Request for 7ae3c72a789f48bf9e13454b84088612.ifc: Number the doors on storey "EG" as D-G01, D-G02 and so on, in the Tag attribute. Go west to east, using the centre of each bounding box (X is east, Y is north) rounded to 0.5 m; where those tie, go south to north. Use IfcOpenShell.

First a look at what the model holds.

```python
import ifcopenshell
import ifcopenshell.util.element
import ifcopenshell.util.placement

model = ifcopenshell.open("7ae3c72a789f48bf9e13454b84088612.ifc")
print(model.schema)
storey = next(s for s in model.by_type("IfcBuildingStorey") if s.Name == "EG")
doors = [e for e in ifcopenshell.util.element.get_decomposition(storey) if e.is_a("IfcDoor")]
for e in sorted(doors, key=lambda e: e.id()):
    origin = ifcopenshell.util.placement.get_local_placement(e.ObjectPlacement)[:3, 3]
    print(e.id(), e.Tag, e.Name, origin.round(2) + 0.0, sep=" | ")
```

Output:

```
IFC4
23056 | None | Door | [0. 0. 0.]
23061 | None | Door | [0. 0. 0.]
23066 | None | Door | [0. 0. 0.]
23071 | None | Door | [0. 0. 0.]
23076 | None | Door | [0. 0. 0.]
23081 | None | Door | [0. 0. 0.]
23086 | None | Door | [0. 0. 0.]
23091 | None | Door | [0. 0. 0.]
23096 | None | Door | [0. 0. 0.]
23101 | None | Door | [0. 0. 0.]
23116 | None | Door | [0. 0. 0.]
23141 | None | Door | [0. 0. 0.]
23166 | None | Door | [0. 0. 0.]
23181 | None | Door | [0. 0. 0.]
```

```python
import ifcopenshell
import ifcopenshell.geom
import ifcopenshell.util.element
import ifcopenshell.util.shape

model = ifcopenshell.open("7ae3c72a789f48bf9e13454b84088612.ifc")
settings = ifcopenshell.geom.settings()
settings.set("use-world-coords", True)


def centre(element):
    shape = ifcopenshell.geom.create_shape(settings, element)
    return ifcopenshell.util.shape.get_bbox_centroid(shape.geometry)


storey = next(s for s in model.by_type("IfcBuildingStorey") if s.Name == "EG")
doors = [e for e in ifcopenshell.util.element.get_decomposition(storey) if e.is_a("IfcDoor")]

# Insertion points can sit at a corner or the storey origin, so sort by the geometry (in metres).
centres = {e: centre(e) for e in doors}
doors.sort(key=lambda e: (round(centres[e][0] / 0.5), centres[e][1]))

for i, e in enumerate(doors, start=1):
    number = f"D-G{i:02d}"
    e.Tag = number
    print(e.id(), number)

model.write("7ae3c72a789f48bf9e13454b84088612_edited.ifc")
```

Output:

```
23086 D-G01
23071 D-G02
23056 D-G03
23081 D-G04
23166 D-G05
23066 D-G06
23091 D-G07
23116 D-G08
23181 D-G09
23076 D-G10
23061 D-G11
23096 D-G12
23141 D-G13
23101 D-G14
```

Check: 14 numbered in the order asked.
